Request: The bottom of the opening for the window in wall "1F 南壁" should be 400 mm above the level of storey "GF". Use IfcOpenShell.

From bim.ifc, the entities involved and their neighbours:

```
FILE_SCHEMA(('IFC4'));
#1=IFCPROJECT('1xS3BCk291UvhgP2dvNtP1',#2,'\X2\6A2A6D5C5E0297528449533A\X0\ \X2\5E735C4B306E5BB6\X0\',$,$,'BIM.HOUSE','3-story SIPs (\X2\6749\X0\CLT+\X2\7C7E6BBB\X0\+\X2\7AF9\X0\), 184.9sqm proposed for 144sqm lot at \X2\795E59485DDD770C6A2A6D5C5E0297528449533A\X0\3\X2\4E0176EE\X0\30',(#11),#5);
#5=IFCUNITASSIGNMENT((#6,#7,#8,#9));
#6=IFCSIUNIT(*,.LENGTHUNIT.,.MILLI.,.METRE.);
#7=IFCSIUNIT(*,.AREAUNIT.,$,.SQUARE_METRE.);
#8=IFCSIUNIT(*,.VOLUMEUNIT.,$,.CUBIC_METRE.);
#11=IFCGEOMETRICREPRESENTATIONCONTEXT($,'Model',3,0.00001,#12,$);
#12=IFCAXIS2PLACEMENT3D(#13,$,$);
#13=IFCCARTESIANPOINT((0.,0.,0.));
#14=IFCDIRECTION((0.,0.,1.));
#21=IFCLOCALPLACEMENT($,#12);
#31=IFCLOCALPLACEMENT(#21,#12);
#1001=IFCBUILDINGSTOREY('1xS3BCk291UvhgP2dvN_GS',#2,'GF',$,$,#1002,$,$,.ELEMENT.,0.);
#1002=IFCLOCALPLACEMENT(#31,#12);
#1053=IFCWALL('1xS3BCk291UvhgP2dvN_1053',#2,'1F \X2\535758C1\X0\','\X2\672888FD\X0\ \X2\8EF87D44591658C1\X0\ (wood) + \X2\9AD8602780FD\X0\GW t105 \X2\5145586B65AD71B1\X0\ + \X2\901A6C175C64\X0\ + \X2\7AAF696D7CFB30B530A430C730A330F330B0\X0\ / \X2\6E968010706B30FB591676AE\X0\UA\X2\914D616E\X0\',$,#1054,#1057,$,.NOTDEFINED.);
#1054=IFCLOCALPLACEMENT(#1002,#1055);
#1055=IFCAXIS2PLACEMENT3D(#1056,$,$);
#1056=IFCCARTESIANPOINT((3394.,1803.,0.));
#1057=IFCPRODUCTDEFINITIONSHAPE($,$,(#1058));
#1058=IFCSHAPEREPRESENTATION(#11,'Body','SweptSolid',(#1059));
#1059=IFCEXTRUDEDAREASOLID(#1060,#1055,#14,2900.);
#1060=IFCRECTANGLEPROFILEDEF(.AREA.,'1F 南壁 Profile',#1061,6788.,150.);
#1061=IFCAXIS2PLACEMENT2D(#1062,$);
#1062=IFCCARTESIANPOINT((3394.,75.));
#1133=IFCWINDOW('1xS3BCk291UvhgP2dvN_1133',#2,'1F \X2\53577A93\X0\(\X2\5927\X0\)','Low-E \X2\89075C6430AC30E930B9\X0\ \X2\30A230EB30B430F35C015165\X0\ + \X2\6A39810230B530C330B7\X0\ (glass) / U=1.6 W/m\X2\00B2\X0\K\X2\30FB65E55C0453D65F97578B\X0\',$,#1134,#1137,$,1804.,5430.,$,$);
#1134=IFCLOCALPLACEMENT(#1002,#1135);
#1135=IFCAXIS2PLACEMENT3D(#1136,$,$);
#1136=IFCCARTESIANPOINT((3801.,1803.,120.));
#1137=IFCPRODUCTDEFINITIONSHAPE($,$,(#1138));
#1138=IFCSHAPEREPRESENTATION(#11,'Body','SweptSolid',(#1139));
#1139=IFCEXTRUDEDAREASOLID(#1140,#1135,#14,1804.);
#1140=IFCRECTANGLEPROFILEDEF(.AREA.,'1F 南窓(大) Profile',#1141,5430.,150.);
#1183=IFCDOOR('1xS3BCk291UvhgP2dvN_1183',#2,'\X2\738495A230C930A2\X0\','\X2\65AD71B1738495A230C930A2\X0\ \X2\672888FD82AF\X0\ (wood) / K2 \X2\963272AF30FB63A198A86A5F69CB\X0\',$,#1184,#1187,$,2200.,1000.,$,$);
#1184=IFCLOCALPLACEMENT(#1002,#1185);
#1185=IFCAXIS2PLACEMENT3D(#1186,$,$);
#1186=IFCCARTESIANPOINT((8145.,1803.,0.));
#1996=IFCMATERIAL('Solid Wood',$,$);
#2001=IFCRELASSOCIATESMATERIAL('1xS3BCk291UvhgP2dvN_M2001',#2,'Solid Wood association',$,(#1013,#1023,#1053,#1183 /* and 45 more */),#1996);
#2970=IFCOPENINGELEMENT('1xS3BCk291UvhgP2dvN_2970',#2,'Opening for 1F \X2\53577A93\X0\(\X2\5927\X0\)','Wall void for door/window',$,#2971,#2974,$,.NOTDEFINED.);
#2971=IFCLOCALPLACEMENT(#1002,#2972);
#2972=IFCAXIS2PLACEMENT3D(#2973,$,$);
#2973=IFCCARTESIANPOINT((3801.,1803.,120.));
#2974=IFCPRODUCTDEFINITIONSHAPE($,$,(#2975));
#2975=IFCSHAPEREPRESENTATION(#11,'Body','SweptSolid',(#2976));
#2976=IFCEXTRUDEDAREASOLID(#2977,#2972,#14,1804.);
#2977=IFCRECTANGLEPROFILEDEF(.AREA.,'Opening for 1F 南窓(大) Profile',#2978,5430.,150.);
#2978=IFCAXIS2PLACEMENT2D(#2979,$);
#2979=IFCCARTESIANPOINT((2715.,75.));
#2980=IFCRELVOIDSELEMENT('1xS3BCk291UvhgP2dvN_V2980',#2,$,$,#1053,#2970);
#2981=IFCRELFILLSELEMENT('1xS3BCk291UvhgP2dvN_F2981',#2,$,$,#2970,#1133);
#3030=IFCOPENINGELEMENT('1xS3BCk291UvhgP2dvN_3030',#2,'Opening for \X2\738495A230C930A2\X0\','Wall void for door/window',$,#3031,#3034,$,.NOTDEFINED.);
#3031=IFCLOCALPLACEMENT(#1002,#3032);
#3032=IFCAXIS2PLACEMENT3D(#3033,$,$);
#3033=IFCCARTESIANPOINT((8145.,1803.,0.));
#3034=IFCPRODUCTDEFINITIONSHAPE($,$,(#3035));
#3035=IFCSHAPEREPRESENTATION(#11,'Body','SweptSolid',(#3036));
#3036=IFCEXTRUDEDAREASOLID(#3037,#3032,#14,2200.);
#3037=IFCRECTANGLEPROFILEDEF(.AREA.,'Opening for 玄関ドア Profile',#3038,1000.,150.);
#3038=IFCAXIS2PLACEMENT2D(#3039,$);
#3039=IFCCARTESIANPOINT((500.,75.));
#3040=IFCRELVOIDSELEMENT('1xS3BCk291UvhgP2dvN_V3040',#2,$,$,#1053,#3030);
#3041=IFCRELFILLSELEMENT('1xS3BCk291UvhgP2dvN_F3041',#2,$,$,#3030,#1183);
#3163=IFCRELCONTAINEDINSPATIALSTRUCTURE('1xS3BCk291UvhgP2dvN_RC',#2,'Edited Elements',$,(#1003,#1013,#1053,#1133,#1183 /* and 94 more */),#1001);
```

```python
import numpy as np
import ifcopenshell
import ifcopenshell.api.geometry
import ifcopenshell.geom
import ifcopenshell.util.element
import ifcopenshell.util.placement
import ifcopenshell.util.shape
import ifcopenshell.util.unit

model = ifcopenshell.open("bim.ifc")
unit_scale = ifcopenshell.util.unit.calculate_unit_scale(model)

window = model.by_id(1133)
opening = window.FillsVoids[0].RelatingOpeningElement
storey = ifcopenshell.util.element.get_container(window, ifc_class="IfcBuildingStorey")
level = ifcopenshell.util.placement.get_local_placement(storey.ObjectPlacement)[2, 3]

# The opening's origin need not be at the sill, so measure its lowest point.
shape = ifcopenshell.geom.create_shape(ifcopenshell.geom.settings(), opening)
bottom = ifcopenshell.util.shape.get_shape_bottom_elevation(shape, shape.geometry) / unit_scale
dz = level + 400.0 - bottom

shift = np.array([0.0, 0.0, dz])
# The window is not placed relative to its opening, so move both.
for product in (opening, window):
    matrix = ifcopenshell.util.placement.get_local_placement(product.ObjectPlacement)
    matrix[:3, 3] += shift
    ifcopenshell.api.geometry.edit_object_placement(model, product=product, matrix=matrix, is_si=False)

print(f"moved by {dz * unit_scale:+.3f} m")

model.write("bim-out.ifc")
```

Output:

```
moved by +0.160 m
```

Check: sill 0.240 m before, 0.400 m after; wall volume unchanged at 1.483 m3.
